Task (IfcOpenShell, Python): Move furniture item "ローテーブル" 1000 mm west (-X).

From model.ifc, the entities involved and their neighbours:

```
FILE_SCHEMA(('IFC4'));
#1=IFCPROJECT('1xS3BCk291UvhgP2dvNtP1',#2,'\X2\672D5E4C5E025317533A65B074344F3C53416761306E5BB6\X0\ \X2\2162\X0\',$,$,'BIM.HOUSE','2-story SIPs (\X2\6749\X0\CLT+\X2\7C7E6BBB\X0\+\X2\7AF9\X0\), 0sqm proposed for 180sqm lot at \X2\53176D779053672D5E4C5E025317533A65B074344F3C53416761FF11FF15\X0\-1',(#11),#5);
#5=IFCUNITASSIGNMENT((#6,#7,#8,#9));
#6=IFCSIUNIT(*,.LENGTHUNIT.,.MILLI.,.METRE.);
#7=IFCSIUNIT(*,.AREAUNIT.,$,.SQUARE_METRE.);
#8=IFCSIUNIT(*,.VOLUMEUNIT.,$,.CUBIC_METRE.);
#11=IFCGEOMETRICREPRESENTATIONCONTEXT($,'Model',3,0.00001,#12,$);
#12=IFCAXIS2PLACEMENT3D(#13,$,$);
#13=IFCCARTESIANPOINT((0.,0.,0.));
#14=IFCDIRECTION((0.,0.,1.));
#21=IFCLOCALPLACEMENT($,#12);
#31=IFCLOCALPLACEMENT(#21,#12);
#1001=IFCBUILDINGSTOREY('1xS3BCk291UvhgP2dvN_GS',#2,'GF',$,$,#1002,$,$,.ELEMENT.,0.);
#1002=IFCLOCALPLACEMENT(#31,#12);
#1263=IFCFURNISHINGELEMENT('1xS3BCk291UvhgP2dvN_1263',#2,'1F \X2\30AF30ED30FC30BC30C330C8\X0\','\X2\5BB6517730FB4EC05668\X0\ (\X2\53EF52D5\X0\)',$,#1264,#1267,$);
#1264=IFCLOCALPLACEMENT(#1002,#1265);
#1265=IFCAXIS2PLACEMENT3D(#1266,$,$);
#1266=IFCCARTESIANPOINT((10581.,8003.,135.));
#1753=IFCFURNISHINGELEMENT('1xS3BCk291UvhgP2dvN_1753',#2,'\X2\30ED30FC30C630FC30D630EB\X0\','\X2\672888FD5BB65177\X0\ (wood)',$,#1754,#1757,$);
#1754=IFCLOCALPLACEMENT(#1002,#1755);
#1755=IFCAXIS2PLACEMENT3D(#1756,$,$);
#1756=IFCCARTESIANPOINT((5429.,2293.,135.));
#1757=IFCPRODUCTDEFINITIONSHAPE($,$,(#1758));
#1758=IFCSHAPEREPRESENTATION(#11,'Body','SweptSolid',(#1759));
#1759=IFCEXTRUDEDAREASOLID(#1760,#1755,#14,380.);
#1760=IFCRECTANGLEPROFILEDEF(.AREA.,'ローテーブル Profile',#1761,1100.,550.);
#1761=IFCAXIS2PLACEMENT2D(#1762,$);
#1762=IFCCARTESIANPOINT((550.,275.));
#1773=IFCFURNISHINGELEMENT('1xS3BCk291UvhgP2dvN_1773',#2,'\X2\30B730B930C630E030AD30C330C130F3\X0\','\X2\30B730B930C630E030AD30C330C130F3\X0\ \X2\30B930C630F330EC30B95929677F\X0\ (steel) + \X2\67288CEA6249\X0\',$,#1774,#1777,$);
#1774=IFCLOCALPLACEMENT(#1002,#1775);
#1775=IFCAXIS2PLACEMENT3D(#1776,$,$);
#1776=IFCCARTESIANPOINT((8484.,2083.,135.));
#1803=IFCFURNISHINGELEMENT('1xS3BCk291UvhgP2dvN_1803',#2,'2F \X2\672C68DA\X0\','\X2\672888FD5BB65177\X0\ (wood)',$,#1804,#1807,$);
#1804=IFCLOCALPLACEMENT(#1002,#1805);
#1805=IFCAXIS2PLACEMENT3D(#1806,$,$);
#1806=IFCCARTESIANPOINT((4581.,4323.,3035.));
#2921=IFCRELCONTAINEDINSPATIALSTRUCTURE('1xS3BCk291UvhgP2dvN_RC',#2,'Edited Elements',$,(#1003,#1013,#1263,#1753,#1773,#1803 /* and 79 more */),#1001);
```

```python
import ifcopenshell
import ifcopenshell.api.geometry
import ifcopenshell.util.placement
import ifcopenshell.util.unit

model = ifcopenshell.open("model.ifc")
unit_scale = ifcopenshell.util.unit.calculate_unit_scale(model)

item = model.by_guid("1xS3BCk291UvhgP2dvN_1753")
matrix = ifcopenshell.util.placement.get_local_placement(item.ObjectPlacement)
matrix[0, 3] -= 1 / unit_scale
ifcopenshell.api.geometry.edit_object_placement(model, product=item, matrix=matrix, is_si=False)

print(ifcopenshell.util.placement.get_local_placement(item.ObjectPlacement).round(3) + 0.0)

model.write("model_rev.ifc")
```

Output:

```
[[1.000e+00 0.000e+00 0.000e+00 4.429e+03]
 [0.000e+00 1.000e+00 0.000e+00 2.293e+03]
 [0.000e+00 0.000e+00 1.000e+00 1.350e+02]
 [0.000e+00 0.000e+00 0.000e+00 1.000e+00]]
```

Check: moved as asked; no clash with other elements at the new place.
